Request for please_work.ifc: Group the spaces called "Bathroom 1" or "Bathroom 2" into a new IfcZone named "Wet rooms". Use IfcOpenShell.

First a look at what the model holds.

```python
import ifcopenshell

model = ifcopenshell.open("please_work.ifc")
print(model.schema)
seen = {}
for space in model.by_type("IfcSpace"):
    seen[space.LongName] = seen.get(space.LongName, 0) + 1
for name, count in sorted(seen.items(), key=str):
    print(count, "x", name)
print("zones:", [z.Name for z in model.by_type("IfcZone")][:20])
```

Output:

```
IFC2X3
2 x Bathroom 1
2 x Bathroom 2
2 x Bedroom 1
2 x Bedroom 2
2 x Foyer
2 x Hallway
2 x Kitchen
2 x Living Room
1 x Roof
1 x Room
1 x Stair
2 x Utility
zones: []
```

```python
import ifcopenshell
import ifcopenshell.api.group
import ifcopenshell.api.root

model = ifcopenshell.open("please_work.ifc")

names = {"Bathroom 1", "Bathroom 2"}
spaces = [s for s in model.by_type("IfcSpace") if s.LongName in names]

zone = ifcopenshell.api.root.create_entity(model, ifc_class="IfcZone", name="Wet rooms")
ifcopenshell.api.group.assign_group(model, products=spaces, group=zone)
print(len(spaces), "spaces in", zone.Name)

model.write("please_work_edited.ifc")
```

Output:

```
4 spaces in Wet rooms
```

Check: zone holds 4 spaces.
